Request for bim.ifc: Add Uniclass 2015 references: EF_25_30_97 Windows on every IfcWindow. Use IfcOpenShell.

First a look at what the model holds.

```python
import ifcopenshell

model = ifcopenshell.open("bim.ifc")
print(model.schema)
print("classifications:", [c.Name for c in model.by_type("IfcClassification")])
for ifc_class in ("IfcDoor", "IfcRoof", "IfcStair", "IfcWall", "IfcWindow"):
    print(ifc_class, len(model.by_type(ifc_class)))
```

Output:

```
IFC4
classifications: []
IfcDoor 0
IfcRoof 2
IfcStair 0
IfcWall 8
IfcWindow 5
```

```python
import ifcopenshell
import ifcopenshell.api.classification

model = ifcopenshell.open("bim.ifc")

system = ifcopenshell.api.classification.add_classification(model, classification="Uniclass 2015")

codes = {
    "IfcWindow": ("EF_25_30_97", "Windows"),
}
for ifc_class, (code, name) in codes.items():
    products = model.by_type(ifc_class)
    ifcopenshell.api.classification.add_reference(
        model, products=products, classification=system, identification=code, name=name
    )
    print(code, len(products))

model.write("bim_rev.ifc")
```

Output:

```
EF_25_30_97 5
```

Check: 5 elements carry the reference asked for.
